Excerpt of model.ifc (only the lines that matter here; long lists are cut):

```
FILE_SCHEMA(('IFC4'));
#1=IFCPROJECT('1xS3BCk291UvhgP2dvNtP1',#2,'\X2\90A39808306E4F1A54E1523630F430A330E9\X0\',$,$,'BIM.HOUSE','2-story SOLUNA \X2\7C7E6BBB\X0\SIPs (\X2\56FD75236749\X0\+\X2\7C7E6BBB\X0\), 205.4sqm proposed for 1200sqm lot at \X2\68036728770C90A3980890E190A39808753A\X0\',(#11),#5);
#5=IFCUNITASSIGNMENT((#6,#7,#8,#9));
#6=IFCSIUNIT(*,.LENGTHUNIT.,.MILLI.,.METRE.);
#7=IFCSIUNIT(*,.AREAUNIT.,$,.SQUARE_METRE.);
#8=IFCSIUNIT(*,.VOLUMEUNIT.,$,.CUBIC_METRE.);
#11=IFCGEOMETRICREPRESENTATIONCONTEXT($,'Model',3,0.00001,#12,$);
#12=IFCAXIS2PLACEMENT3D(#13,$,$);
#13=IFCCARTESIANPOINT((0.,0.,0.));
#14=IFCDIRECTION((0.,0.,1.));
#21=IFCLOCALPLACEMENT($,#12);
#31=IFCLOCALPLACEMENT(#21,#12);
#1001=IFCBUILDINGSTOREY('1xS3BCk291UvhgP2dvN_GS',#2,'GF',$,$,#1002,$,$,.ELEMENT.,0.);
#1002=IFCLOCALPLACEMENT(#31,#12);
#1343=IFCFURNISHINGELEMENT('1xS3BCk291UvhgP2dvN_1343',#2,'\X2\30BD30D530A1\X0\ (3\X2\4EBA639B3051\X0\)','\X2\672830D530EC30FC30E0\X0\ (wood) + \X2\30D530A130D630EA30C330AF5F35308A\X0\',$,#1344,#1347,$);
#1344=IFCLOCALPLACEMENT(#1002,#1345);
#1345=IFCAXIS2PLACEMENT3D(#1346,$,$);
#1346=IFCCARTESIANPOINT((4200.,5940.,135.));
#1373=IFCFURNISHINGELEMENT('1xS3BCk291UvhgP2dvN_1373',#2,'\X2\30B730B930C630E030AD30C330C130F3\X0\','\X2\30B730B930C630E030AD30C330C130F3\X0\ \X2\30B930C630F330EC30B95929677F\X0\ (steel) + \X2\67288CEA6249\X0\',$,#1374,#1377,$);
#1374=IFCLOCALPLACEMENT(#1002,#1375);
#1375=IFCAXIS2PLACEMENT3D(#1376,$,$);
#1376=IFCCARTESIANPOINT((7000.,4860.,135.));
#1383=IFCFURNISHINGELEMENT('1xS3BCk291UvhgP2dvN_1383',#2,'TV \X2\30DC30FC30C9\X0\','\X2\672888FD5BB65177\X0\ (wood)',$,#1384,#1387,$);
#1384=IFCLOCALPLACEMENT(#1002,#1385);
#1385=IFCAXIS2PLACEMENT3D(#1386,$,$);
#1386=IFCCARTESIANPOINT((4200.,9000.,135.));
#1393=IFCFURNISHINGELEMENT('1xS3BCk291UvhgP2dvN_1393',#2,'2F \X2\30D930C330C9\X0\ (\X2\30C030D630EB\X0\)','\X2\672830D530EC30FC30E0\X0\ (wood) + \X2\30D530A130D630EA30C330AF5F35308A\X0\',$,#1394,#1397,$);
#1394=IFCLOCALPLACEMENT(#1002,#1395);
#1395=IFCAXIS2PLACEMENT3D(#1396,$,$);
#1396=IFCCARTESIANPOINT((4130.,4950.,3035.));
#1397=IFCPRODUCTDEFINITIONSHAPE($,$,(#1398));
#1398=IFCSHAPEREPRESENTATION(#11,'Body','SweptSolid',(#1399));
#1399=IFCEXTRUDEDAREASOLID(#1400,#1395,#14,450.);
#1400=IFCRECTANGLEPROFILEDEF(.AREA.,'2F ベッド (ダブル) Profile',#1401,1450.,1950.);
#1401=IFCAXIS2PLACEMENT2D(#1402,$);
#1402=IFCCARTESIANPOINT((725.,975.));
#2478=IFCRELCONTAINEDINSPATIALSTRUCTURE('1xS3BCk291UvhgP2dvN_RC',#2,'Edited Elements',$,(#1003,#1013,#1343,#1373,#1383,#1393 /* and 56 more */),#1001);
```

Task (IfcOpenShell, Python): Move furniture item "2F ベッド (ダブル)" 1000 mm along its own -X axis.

```python
import ifcopenshell
import ifcopenshell.api.geometry
import ifcopenshell.util.placement

model = ifcopenshell.open("model.ifc")

item = model.by_guid("1xS3BCk291UvhgP2dvN_1393")
matrix = ifcopenshell.util.placement.get_local_placement(item.ObjectPlacement)
matrix[:3, 3] -= matrix[:3, 0] * 1000.0
ifcopenshell.api.geometry.edit_object_placement(model, product=item, matrix=matrix, is_si=False)

print(ifcopenshell.util.placement.get_local_placement(item.ObjectPlacement).round(3) + 0.0)

model.write("model_updated.ifc")
```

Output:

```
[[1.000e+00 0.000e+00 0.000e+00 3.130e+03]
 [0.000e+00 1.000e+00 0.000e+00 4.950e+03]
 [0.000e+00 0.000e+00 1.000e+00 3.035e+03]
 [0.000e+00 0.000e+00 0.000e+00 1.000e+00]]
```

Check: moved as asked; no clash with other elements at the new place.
